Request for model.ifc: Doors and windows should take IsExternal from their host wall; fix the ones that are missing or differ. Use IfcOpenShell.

First a look at what the model holds.

```python
import ifcopenshell
import ifcopenshell.util.element

model = ifcopenshell.open("model.ifc")
print(model.schema)
seen = {}
for e in model.by_type("IfcDoor") + model.by_type("IfcWindow"):
    if not e.FillsVoids:
        continue
    host = e.FillsVoids[0].RelatingOpeningElement.VoidsElements[0].RelatingBuildingElement
    own = ifcopenshell.util.element.get_pset(e, f"Pset_{e.is_a()[3:].removesuffix('StandardCase')}Common", "IsExternal")
    wall = ifcopenshell.util.element.get_pset(host, "Pset_WallCommon", "IsExternal")
    seen[e.is_a(), own, wall] = seen.get((e.is_a(), own, wall), 0) + 1
for (cls, own, wall), count in sorted(seen.items(), key=str):
    print(count, cls, "IsExternal:", own, "| host wall:", wall)
```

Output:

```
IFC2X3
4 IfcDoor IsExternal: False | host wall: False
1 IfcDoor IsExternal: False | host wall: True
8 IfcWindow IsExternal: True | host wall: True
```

```python
import ifcopenshell
import ifcopenshell.api.pset
import ifcopenshell.util.element

model = ifcopenshell.open("model.ifc")

count = 0
for ifc_class, pset_name in (("IfcDoor", "Pset_DoorCommon"), ("IfcWindow", "Pset_WindowCommon")):
    for e in model.by_type(ifc_class):
        if not e.FillsVoids:
            continue
        host = e.FillsVoids[0].RelatingOpeningElement.VoidsElements[0].RelatingBuildingElement
        external = ifcopenshell.util.element.get_pset(host, "Pset_WallCommon", "IsExternal")
        if external is None or ifcopenshell.util.element.get_pset(e, pset_name, "IsExternal") == external:
            continue
        pset = ifcopenshell.api.pset.add_pset(model, product=e, name=pset_name)
        ifcopenshell.api.pset.edit_pset(model, pset=pset, properties={"IsExternal": external})
        count += 1

print(count, "updated")

model.write("model_updated.ifc")
```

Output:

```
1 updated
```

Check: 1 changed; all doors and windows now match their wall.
